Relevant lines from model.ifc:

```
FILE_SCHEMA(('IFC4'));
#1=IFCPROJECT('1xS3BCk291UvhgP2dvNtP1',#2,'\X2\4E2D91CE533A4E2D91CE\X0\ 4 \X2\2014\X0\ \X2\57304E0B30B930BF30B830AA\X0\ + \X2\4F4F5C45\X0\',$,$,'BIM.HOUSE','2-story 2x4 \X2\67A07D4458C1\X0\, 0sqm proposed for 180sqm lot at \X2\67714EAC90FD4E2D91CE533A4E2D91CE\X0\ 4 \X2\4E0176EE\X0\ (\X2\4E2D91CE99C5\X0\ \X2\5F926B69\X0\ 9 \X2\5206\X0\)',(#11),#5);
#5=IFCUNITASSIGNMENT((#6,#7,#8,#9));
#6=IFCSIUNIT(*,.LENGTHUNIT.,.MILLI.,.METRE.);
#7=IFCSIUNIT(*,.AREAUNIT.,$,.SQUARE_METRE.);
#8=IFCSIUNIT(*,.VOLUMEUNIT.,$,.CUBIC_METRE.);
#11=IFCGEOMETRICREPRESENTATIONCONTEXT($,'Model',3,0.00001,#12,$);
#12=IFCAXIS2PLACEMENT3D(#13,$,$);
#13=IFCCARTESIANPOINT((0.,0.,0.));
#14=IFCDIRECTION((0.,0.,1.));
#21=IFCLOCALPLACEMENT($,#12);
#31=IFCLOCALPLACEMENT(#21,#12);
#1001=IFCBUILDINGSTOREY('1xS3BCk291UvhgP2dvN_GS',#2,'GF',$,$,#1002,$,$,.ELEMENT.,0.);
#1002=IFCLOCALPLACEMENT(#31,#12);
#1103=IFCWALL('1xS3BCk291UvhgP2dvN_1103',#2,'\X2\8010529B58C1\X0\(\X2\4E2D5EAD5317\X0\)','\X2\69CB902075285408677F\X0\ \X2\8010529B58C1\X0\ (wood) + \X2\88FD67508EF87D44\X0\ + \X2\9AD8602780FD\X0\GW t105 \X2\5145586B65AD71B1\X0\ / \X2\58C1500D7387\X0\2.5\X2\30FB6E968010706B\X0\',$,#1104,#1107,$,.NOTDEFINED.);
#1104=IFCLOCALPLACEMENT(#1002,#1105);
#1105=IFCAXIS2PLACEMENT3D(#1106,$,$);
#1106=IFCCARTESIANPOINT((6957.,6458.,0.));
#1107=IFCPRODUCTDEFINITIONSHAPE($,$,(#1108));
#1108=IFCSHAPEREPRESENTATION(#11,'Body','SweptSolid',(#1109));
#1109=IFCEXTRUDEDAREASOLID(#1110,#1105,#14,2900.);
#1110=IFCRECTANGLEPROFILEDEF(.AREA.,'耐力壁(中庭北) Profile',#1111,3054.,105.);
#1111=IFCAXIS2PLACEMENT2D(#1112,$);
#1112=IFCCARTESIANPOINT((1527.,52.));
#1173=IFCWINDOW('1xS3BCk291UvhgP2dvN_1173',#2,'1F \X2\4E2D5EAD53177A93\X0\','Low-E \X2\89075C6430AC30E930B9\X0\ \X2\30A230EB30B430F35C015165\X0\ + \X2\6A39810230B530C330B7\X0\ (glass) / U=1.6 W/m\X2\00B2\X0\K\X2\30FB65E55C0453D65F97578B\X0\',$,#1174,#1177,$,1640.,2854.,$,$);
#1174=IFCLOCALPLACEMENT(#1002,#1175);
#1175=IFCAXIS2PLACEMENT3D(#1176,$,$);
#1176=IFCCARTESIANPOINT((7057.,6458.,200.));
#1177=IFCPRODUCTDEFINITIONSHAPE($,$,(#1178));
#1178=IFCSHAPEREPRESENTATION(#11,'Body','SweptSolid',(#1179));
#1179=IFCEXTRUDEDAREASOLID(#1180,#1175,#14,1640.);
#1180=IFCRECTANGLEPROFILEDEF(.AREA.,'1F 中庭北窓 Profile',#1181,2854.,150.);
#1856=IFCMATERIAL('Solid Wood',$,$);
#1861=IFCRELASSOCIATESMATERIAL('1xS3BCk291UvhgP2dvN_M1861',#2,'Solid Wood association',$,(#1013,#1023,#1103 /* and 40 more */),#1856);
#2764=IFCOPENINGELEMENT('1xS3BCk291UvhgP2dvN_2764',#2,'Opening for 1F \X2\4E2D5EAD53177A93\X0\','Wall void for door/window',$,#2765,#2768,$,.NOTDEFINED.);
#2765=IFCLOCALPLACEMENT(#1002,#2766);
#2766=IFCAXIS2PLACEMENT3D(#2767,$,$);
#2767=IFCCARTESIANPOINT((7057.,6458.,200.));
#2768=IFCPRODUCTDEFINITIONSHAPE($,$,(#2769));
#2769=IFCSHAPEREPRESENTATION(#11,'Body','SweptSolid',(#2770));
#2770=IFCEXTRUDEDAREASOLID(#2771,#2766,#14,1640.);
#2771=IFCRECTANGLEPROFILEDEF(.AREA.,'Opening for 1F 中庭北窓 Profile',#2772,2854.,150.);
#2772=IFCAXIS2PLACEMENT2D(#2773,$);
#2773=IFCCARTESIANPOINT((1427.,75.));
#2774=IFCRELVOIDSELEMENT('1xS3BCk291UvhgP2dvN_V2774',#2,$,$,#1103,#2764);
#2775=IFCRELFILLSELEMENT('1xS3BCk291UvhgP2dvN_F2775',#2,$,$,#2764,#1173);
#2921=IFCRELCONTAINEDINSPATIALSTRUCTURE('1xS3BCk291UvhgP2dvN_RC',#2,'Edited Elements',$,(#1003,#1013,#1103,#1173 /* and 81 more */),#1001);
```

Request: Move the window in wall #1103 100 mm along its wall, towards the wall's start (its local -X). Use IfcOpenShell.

```python
import ifcopenshell
import ifcopenshell.api.geometry
import ifcopenshell.util.placement

model = ifcopenshell.open("model.ifc")

window = model.by_id(1173)
opening = window.FillsVoids[0].RelatingOpeningElement
wall = opening.VoidsElements[0].RelatingBuildingElement

wall_matrix = ifcopenshell.util.placement.get_local_placement(wall.ObjectPlacement)
shift = wall_matrix[:3, 0] * -100.0
before = ifcopenshell.util.placement.get_local_placement(window.ObjectPlacement)[:3, 3].copy()

# The window is not placed relative to its opening, so move both.
for product in (opening, window):
    matrix = ifcopenshell.util.placement.get_local_placement(product.ObjectPlacement)
    matrix[:3, 3] += shift
    ifcopenshell.api.geometry.edit_object_placement(model, product=product, matrix=matrix, is_si=False)

after = ifcopenshell.util.placement.get_local_placement(window.ObjectPlacement)[:3, 3]
print("window moved by", (after - before).round(3) + 0.0)

model.write("model-out.ifc")
```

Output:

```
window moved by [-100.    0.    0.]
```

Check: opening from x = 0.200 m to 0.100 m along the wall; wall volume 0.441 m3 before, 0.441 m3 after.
